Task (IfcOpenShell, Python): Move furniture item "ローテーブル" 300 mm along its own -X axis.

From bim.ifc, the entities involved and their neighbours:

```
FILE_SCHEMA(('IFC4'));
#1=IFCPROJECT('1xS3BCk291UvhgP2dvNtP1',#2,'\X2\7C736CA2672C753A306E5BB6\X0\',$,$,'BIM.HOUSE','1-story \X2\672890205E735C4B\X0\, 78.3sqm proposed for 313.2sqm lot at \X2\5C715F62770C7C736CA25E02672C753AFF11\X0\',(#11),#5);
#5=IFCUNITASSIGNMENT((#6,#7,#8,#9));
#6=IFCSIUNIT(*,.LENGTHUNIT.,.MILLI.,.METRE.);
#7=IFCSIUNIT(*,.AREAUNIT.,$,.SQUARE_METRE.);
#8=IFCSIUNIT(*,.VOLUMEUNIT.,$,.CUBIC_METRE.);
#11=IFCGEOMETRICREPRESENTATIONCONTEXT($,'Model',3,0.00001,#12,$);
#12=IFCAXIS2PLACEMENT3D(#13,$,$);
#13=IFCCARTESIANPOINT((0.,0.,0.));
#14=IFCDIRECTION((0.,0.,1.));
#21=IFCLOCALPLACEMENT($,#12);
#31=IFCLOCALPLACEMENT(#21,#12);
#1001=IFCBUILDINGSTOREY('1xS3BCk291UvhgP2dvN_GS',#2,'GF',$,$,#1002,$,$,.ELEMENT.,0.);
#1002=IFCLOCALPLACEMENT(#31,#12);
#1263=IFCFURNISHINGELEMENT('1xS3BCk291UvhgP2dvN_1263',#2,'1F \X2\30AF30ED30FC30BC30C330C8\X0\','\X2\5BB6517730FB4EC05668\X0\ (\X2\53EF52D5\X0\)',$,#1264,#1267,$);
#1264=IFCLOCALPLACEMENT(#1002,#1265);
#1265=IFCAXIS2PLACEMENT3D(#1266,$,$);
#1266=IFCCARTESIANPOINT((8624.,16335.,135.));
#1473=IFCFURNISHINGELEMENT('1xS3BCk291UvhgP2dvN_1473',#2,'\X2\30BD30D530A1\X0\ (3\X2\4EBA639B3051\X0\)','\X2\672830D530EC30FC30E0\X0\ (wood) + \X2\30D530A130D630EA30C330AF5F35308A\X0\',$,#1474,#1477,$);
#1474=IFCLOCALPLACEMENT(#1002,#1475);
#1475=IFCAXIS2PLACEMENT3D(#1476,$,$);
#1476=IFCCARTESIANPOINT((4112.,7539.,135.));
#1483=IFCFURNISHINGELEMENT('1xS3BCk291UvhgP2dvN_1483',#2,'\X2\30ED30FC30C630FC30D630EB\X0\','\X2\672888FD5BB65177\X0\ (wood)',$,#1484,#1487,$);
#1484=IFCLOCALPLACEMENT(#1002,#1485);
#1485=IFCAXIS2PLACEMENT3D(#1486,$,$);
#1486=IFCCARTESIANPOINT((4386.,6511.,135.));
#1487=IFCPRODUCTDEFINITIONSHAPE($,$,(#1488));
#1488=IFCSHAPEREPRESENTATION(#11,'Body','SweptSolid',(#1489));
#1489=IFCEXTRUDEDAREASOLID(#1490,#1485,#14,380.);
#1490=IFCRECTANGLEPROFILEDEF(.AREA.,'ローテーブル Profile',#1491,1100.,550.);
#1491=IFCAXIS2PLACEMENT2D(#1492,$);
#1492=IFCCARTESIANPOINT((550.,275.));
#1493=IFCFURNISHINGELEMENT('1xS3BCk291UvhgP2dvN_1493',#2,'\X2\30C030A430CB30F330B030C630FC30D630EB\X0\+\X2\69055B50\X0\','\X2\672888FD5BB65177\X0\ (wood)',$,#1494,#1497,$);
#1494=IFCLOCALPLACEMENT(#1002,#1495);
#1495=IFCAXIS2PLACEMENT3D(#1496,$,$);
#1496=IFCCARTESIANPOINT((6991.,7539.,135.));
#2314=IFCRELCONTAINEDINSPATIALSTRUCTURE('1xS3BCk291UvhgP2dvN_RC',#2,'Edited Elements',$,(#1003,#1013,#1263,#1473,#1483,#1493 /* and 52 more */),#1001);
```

```python
import ifcopenshell
import ifcopenshell.api.geometry
import ifcopenshell.util.placement

model = ifcopenshell.open("bim.ifc")

item = model.by_id(1483)
matrix = ifcopenshell.util.placement.get_local_placement(item.ObjectPlacement)
matrix[:3, 3] -= matrix[:3, 0] * 300.0
ifcopenshell.api.geometry.edit_object_placement(model, product=item, matrix=matrix, is_si=False)

print(ifcopenshell.util.placement.get_local_placement(item.ObjectPlacement).round(3) + 0.0)

model.write("bim_edited.ifc")
```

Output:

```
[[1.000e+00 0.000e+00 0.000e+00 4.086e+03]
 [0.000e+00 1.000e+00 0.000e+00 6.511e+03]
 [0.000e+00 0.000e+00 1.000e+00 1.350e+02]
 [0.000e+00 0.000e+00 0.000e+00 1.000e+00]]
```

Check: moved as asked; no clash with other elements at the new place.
